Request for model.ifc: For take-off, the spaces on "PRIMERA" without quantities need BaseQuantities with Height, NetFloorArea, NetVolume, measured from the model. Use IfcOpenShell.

First a look at what the model holds.

```python
import ifcopenshell
import ifcopenshell.util.element
import ifcopenshell.util.unit

model = ifcopenshell.open("model.ifc")
print(model.schema)
for unit_type in ("LENGTHUNIT", "AREAUNIT", "VOLUMEUNIT"):
    print(unit_type, ifcopenshell.util.unit.calculate_unit_scale(model, unit_type))
storey = next(s for s in model.by_type("IfcBuildingStorey") if s.Name == "PRIMERA")
spaces = [e for e in ifcopenshell.util.element.get_decomposition(storey) if e.is_a("IfcSpace")]
for e in sorted(spaces, key=lambda e: e.id()):
    print(e.id(), e.is_a(), e.Name, list(ifcopenshell.util.element.get_psets(e, qtos_only=True)), sep=" | ")
```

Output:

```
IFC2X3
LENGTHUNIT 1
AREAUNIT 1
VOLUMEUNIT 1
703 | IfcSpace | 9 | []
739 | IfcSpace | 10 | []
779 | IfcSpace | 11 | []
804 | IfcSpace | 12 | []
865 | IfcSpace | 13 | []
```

```python
import ifcopenshell
import ifcopenshell.api.pset
import ifcopenshell.geom
import ifcopenshell.util.element
import ifcopenshell.util.shape
import ifcopenshell.util.unit

model = ifcopenshell.open("model.ifc")
unit_scale = ifcopenshell.util.unit.calculate_unit_scale(model)
area_scale = ifcopenshell.util.unit.calculate_unit_scale(model, "AREAUNIT")
volume_scale = ifcopenshell.util.unit.calculate_unit_scale(model, "VOLUMEUNIT")
settings = ifcopenshell.geom.settings()

storey = next(s for s in model.by_type("IfcBuildingStorey") if s.Name == "PRIMERA")
spaces = [e for e in ifcopenshell.util.element.get_decomposition(storey) if e.is_a("IfcSpace")]

for e in sorted(spaces, key=lambda e: e.id()):
    if ifcopenshell.util.element.get_psets(e, qtos_only=True, should_inherit=False):
        continue
    # Geometry comes back in metres, in the element's own axes.
    shape = ifcopenshell.geom.create_shape(settings, e)
    values = {
        "Height": ifcopenshell.util.shape.get_z(shape.geometry) / unit_scale,
        "NetFloorArea": ifcopenshell.util.shape.get_footprint_area(shape.geometry) / area_scale,
        "NetVolume": ifcopenshell.util.shape.get_volume(shape.geometry) / volume_scale,
    }
    qto = ifcopenshell.api.pset.add_qto(model, product=e, name="BaseQuantities")
    ifcopenshell.api.pset.edit_qto(model, qto=qto, properties=values)
    print(e.id(), {k: round(v, 3) for k, v in values.items()})

model.write("model_rev.ifc")
```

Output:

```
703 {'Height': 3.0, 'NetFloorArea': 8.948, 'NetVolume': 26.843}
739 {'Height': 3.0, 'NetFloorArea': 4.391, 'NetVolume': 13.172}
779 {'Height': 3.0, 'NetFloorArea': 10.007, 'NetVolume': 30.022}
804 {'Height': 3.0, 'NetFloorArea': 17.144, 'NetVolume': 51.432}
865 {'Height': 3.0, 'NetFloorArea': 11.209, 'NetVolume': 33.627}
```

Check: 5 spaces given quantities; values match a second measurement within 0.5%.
